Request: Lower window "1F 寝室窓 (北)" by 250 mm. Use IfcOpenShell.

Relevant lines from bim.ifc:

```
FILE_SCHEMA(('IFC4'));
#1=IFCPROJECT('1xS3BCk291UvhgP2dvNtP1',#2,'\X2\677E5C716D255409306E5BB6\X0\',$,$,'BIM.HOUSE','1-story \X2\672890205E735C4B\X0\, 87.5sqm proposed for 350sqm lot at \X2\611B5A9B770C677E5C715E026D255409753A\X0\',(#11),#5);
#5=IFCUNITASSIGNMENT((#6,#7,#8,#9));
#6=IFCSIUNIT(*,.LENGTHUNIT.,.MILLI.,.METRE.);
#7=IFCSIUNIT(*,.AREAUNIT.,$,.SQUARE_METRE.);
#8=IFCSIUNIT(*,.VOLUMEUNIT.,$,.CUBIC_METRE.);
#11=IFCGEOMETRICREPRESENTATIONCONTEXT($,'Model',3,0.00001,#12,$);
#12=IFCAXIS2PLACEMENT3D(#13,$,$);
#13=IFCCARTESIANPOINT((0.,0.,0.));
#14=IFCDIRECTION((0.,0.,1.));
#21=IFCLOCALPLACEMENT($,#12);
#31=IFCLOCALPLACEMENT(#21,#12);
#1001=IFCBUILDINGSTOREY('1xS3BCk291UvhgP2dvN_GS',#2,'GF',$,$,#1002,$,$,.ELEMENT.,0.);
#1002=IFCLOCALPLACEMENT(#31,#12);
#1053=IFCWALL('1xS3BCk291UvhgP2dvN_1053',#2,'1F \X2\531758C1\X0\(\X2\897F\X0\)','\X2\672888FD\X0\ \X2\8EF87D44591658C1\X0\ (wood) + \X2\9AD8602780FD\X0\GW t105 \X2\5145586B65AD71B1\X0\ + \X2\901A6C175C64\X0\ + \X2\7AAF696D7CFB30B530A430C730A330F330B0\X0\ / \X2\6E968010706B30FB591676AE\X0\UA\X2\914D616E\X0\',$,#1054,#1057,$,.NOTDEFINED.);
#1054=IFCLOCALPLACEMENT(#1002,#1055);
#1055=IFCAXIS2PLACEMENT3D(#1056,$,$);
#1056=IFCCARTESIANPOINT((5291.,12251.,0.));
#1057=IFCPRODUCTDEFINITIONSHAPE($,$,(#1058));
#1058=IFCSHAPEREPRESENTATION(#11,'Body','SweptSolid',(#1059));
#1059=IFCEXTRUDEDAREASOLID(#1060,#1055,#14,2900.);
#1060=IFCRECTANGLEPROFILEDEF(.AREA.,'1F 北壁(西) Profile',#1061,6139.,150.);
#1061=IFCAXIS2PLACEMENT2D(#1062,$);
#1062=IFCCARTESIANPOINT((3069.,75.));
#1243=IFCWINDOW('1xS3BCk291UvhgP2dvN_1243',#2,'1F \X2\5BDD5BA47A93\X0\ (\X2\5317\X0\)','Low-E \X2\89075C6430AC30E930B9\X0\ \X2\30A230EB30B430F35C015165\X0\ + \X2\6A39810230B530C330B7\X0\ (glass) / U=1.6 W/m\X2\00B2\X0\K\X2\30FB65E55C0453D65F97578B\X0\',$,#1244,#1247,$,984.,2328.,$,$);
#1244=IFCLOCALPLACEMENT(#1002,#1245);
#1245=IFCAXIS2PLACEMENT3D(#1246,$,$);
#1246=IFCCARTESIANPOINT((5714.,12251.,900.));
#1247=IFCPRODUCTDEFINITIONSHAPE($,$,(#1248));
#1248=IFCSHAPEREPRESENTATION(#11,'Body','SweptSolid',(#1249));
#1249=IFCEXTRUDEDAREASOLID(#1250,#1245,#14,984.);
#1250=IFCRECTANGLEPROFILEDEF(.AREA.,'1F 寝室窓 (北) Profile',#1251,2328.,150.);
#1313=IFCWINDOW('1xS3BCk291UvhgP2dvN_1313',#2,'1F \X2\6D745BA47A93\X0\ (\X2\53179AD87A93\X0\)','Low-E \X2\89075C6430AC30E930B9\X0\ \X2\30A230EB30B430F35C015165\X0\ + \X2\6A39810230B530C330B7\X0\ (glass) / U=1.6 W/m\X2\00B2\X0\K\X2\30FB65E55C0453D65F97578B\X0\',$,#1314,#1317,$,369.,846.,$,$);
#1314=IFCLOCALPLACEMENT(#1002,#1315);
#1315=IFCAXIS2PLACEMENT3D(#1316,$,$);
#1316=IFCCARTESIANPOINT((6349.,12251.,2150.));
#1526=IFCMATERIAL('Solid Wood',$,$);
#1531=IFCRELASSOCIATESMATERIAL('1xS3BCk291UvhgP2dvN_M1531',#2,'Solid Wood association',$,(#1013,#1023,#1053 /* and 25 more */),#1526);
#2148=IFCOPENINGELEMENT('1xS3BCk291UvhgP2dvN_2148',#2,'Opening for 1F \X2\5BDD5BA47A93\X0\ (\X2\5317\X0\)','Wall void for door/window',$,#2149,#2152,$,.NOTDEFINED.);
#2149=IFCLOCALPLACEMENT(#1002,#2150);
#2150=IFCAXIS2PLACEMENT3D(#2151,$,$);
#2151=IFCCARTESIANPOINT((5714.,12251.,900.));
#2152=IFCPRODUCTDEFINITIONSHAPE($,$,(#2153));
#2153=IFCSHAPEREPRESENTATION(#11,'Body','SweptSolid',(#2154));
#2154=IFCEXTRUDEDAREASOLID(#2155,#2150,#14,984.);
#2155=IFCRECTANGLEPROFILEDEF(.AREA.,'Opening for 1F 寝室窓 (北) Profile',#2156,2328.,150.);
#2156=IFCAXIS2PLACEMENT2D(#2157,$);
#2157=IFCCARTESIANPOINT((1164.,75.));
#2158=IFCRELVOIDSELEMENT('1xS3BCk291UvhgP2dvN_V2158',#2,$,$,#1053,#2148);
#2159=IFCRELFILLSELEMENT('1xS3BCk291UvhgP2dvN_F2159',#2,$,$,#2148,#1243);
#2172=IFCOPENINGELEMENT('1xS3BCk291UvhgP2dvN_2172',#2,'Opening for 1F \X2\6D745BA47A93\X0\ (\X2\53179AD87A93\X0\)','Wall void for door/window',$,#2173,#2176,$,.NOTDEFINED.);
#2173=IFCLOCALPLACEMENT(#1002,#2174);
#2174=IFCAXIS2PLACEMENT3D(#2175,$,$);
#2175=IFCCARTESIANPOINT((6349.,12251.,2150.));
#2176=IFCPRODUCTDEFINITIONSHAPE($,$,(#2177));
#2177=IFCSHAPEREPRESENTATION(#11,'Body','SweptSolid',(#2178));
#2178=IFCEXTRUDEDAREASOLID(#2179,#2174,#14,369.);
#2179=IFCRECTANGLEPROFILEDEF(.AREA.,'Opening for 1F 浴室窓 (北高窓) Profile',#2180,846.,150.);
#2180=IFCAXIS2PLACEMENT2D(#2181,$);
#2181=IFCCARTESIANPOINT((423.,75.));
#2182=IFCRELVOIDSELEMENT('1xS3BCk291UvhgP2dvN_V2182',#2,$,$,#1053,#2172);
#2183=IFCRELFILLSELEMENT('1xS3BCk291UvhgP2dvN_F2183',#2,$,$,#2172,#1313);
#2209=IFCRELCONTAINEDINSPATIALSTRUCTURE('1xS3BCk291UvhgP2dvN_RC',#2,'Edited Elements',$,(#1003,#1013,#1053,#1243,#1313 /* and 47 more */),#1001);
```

```python
import numpy as np
import ifcopenshell
import ifcopenshell.api.geometry
import ifcopenshell.util.placement
import ifcopenshell.util.unit

model = ifcopenshell.open("bim.ifc")
unit_scale = ifcopenshell.util.unit.calculate_unit_scale(model)

window = model.by_guid("1xS3BCk291UvhgP2dvN_1243")
opening = window.FillsVoids[0].RelatingOpeningElement
dz = -250.0

shift = np.array([0.0, 0.0, dz])
# The window is not placed relative to its opening, so move both.
for product in (opening, window):
    matrix = ifcopenshell.util.placement.get_local_placement(product.ObjectPlacement)
    matrix[:3, 3] += shift
    ifcopenshell.api.geometry.edit_object_placement(model, product=product, matrix=matrix, is_si=False)

print(f"moved by {dz * unit_scale:+.3f} m")

model.write("bim-out.ifc")
```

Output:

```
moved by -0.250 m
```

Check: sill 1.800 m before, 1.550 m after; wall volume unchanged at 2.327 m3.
